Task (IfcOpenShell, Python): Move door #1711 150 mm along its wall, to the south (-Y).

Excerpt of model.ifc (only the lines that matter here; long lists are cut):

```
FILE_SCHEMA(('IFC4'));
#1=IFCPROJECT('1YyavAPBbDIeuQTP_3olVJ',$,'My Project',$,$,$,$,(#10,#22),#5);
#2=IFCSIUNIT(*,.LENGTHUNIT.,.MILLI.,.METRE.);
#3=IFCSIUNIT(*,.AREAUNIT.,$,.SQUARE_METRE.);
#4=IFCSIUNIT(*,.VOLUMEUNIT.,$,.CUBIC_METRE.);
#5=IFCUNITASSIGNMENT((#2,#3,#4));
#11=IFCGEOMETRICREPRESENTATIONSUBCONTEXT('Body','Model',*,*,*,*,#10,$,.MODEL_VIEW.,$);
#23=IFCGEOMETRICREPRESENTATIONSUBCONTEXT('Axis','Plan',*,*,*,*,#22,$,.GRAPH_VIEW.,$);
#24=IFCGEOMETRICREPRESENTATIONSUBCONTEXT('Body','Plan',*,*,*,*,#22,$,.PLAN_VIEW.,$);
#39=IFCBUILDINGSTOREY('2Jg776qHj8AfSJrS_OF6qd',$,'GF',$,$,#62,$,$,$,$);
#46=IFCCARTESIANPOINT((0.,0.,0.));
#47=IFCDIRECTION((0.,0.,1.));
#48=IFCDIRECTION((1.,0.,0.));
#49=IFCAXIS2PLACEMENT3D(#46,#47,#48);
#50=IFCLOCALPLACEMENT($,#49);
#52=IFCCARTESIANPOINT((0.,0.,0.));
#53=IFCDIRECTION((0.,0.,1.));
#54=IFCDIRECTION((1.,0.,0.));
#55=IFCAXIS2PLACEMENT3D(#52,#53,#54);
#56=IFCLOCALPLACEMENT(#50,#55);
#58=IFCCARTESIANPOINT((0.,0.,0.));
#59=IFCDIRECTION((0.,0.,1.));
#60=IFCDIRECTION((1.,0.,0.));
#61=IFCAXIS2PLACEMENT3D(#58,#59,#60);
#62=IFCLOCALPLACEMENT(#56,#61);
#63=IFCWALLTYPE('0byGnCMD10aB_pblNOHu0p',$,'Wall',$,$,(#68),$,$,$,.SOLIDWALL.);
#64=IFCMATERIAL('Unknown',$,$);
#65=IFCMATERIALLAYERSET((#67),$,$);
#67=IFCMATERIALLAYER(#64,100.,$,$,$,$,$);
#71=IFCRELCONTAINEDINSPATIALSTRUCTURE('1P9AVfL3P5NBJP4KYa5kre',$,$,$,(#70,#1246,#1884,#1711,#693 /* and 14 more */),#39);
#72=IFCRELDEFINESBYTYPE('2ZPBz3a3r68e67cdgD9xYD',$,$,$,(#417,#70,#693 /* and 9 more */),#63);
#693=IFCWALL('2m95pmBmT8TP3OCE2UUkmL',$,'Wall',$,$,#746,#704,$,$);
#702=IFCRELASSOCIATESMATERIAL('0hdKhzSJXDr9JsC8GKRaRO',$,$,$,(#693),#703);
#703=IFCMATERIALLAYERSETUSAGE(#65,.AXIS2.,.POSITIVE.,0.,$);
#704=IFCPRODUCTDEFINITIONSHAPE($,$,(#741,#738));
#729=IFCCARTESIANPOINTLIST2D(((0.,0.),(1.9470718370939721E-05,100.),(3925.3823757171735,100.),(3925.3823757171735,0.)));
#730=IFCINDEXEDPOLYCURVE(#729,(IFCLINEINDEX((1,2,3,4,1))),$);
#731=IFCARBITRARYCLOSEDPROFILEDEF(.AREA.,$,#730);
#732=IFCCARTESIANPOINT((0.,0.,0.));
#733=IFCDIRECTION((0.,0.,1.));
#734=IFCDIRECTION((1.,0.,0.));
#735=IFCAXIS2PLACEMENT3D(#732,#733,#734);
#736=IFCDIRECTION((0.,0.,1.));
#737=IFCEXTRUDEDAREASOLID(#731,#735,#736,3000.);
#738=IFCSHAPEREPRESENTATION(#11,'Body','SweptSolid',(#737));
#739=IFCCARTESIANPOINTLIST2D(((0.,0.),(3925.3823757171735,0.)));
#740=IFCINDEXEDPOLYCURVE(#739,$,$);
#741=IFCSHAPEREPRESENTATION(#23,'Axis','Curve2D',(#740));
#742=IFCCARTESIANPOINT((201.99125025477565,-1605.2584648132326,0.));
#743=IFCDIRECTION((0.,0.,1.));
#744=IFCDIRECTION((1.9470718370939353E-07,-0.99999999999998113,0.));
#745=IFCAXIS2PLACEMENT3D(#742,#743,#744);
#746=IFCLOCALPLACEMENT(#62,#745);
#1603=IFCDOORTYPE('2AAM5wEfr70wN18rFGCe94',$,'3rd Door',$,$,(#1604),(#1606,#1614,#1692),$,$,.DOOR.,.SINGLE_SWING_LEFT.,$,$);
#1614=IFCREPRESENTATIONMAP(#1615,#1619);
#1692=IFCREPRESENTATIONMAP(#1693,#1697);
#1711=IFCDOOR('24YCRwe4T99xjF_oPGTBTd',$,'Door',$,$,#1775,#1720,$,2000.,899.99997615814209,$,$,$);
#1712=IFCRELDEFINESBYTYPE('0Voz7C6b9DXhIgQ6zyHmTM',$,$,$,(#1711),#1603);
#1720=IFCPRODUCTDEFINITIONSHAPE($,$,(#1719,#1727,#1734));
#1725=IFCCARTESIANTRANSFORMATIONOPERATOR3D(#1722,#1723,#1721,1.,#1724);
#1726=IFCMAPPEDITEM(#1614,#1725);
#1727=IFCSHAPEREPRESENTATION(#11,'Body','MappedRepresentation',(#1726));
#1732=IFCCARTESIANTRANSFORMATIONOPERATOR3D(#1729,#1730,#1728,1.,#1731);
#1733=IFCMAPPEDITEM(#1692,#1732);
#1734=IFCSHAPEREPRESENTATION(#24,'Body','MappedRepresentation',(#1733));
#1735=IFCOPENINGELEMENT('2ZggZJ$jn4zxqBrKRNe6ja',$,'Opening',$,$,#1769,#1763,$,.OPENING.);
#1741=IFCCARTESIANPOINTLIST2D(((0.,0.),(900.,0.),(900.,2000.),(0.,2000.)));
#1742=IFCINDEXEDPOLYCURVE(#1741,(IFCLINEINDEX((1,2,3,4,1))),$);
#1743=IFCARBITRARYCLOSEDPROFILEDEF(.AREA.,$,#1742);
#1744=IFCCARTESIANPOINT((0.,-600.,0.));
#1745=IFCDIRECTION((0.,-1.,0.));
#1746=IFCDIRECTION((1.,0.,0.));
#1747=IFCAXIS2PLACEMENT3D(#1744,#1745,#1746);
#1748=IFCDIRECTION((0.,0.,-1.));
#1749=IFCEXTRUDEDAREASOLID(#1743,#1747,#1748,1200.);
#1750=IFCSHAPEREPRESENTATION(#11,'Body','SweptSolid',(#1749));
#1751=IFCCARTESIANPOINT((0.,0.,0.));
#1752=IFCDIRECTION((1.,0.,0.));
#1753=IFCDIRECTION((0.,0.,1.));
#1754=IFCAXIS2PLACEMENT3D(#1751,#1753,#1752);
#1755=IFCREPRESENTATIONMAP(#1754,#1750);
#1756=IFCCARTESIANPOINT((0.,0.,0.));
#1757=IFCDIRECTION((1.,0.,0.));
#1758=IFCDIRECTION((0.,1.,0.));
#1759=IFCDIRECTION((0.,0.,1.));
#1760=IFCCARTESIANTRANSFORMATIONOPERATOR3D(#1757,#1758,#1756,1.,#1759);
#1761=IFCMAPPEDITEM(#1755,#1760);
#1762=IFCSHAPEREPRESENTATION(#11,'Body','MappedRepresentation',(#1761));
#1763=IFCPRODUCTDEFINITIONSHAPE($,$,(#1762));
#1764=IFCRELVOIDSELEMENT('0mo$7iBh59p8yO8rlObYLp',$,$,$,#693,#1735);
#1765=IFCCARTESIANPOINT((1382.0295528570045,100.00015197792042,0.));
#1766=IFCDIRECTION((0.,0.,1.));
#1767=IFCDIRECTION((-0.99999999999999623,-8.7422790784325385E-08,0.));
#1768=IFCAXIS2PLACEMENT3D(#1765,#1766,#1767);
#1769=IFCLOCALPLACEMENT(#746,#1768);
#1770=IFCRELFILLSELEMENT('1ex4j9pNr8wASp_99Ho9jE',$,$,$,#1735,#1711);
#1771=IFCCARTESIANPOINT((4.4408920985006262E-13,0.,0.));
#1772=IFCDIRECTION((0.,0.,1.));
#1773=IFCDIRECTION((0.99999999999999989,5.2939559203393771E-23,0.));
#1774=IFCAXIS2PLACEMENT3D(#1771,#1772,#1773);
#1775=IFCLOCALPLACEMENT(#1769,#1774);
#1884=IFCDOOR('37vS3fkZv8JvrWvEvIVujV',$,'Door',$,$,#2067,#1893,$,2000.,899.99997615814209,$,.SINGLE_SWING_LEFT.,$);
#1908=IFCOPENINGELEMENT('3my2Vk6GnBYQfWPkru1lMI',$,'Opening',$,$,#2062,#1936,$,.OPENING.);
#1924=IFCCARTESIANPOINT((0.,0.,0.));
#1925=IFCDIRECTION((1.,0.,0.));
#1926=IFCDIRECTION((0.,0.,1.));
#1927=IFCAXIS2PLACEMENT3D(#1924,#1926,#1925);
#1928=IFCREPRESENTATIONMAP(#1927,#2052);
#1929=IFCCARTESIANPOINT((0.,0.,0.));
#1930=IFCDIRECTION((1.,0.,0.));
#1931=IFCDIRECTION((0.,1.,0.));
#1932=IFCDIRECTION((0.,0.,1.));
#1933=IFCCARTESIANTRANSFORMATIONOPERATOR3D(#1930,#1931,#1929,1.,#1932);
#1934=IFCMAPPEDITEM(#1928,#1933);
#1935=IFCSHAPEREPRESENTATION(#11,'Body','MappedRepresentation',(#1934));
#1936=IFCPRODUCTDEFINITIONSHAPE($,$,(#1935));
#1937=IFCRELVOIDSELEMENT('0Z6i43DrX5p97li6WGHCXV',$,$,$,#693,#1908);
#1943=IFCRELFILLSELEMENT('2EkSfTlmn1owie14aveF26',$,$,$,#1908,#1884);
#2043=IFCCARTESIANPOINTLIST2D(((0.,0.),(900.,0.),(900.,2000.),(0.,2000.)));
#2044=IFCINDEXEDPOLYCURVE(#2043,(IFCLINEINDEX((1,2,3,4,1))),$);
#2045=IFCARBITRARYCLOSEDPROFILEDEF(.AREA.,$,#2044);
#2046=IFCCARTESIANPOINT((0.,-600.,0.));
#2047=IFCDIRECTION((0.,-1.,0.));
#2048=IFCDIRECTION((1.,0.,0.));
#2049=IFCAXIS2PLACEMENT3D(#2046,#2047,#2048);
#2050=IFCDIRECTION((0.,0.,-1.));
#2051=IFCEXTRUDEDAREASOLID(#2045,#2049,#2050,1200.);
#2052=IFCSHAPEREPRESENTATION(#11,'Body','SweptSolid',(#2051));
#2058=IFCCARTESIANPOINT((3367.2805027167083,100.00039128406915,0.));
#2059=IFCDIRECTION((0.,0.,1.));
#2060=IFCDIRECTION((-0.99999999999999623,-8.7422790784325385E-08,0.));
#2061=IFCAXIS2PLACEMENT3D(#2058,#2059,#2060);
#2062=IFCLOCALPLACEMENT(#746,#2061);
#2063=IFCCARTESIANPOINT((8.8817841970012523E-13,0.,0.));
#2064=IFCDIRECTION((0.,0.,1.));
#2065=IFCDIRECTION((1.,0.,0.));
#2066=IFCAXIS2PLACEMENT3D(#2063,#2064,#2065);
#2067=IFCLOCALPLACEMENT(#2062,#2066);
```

```python
import ifcopenshell
import ifcopenshell.api.geometry
import ifcopenshell.util.placement
import ifcopenshell.util.unit

model = ifcopenshell.open("model.ifc")
unit_scale = ifcopenshell.util.unit.calculate_unit_scale(model)

door = model.by_guid("24YCRwe4T99xjF_oPGTBTd")
opening = door.FillsVoids[0].RelatingOpeningElement
wall = opening.VoidsElements[0].RelatingBuildingElement

wall_matrix = ifcopenshell.util.placement.get_local_placement(wall.ObjectPlacement)
shift = wall_matrix[:3, 0] * 0.15 / unit_scale
before = ifcopenshell.util.placement.get_local_placement(door.ObjectPlacement)[:3, 3].copy()

# The door is placed relative to its opening, so it follows when the opening moves.
matrix = ifcopenshell.util.placement.get_local_placement(opening.ObjectPlacement)
matrix[:3, 3] += shift
ifcopenshell.api.geometry.edit_object_placement(
    model, product=opening, matrix=matrix, is_si=False, should_transform_children=True
)

after = ifcopenshell.util.placement.get_local_placement(door.ObjectPlacement)[:3, 3]
print("door moved by", (after - before).round(3) + 0.0)

model.write("model_v2.ifc")
```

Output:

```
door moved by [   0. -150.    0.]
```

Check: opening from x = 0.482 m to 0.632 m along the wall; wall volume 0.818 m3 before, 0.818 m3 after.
